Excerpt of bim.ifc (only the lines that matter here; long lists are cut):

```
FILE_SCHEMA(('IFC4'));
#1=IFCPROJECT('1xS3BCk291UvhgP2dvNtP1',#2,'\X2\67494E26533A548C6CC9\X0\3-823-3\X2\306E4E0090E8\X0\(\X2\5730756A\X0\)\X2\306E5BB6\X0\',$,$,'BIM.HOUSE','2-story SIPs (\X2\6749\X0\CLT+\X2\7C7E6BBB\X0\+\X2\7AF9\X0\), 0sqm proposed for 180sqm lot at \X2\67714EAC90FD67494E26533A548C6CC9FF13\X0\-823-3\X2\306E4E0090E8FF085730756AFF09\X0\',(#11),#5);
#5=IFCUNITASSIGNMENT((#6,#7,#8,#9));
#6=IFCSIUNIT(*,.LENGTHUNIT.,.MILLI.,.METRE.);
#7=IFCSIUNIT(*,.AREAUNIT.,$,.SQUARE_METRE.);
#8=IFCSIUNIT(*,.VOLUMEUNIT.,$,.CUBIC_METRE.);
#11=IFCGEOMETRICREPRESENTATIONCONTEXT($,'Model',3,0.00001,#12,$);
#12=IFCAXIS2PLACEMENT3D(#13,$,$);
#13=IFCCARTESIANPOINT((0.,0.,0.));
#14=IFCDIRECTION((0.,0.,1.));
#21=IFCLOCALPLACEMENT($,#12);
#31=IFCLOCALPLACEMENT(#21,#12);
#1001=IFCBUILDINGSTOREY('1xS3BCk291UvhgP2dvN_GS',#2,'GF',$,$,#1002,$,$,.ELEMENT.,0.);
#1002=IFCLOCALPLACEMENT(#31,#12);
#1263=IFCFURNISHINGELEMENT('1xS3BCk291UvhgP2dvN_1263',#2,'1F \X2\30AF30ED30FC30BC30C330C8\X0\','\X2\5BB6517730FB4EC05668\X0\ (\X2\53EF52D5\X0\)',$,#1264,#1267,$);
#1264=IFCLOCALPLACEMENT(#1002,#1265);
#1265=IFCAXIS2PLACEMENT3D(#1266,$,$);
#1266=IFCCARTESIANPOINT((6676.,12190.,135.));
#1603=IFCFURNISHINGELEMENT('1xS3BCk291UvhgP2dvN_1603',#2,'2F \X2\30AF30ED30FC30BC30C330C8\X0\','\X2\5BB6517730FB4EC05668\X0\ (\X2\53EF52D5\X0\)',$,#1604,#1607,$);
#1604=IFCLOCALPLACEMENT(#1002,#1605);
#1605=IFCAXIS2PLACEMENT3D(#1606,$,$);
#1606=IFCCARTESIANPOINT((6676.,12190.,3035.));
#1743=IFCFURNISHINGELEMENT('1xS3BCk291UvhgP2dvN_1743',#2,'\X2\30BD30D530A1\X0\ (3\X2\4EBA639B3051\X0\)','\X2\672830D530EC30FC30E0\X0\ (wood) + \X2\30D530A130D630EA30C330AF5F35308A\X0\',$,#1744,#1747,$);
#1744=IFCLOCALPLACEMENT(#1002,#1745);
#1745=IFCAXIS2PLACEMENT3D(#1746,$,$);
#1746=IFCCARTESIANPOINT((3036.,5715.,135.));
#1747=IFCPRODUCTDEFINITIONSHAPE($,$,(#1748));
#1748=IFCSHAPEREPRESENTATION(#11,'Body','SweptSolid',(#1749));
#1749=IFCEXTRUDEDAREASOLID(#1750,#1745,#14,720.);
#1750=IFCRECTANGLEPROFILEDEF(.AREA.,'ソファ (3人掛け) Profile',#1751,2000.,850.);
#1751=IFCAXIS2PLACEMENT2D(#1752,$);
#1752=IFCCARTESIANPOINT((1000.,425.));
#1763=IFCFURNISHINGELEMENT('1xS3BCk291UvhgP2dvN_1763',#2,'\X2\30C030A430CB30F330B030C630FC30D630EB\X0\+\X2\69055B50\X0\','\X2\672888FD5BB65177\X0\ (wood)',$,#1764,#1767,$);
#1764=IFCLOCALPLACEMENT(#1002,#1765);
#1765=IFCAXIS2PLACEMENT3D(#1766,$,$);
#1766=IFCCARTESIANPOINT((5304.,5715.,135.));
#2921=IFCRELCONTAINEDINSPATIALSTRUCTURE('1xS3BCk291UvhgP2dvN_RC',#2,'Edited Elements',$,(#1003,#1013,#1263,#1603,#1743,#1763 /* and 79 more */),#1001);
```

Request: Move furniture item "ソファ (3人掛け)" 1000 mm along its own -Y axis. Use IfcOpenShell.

```python
import ifcopenshell
import ifcopenshell.api.geometry
import ifcopenshell.util.placement
import ifcopenshell.util.unit

model = ifcopenshell.open("bim.ifc")
unit_scale = ifcopenshell.util.unit.calculate_unit_scale(model)

item = model.by_id(1743)
matrix = ifcopenshell.util.placement.get_local_placement(item.ObjectPlacement)
matrix[:3, 3] -= matrix[:3, 1] * 1 / unit_scale
ifcopenshell.api.geometry.edit_object_placement(model, product=item, matrix=matrix, is_si=False)

print(ifcopenshell.util.placement.get_local_placement(item.ObjectPlacement).round(3) + 0.0)

model.write("bim-out.ifc")
```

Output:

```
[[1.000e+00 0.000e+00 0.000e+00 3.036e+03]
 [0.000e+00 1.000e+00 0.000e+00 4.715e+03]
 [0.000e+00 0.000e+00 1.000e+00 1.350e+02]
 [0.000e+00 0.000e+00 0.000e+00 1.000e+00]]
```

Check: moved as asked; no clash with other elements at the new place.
